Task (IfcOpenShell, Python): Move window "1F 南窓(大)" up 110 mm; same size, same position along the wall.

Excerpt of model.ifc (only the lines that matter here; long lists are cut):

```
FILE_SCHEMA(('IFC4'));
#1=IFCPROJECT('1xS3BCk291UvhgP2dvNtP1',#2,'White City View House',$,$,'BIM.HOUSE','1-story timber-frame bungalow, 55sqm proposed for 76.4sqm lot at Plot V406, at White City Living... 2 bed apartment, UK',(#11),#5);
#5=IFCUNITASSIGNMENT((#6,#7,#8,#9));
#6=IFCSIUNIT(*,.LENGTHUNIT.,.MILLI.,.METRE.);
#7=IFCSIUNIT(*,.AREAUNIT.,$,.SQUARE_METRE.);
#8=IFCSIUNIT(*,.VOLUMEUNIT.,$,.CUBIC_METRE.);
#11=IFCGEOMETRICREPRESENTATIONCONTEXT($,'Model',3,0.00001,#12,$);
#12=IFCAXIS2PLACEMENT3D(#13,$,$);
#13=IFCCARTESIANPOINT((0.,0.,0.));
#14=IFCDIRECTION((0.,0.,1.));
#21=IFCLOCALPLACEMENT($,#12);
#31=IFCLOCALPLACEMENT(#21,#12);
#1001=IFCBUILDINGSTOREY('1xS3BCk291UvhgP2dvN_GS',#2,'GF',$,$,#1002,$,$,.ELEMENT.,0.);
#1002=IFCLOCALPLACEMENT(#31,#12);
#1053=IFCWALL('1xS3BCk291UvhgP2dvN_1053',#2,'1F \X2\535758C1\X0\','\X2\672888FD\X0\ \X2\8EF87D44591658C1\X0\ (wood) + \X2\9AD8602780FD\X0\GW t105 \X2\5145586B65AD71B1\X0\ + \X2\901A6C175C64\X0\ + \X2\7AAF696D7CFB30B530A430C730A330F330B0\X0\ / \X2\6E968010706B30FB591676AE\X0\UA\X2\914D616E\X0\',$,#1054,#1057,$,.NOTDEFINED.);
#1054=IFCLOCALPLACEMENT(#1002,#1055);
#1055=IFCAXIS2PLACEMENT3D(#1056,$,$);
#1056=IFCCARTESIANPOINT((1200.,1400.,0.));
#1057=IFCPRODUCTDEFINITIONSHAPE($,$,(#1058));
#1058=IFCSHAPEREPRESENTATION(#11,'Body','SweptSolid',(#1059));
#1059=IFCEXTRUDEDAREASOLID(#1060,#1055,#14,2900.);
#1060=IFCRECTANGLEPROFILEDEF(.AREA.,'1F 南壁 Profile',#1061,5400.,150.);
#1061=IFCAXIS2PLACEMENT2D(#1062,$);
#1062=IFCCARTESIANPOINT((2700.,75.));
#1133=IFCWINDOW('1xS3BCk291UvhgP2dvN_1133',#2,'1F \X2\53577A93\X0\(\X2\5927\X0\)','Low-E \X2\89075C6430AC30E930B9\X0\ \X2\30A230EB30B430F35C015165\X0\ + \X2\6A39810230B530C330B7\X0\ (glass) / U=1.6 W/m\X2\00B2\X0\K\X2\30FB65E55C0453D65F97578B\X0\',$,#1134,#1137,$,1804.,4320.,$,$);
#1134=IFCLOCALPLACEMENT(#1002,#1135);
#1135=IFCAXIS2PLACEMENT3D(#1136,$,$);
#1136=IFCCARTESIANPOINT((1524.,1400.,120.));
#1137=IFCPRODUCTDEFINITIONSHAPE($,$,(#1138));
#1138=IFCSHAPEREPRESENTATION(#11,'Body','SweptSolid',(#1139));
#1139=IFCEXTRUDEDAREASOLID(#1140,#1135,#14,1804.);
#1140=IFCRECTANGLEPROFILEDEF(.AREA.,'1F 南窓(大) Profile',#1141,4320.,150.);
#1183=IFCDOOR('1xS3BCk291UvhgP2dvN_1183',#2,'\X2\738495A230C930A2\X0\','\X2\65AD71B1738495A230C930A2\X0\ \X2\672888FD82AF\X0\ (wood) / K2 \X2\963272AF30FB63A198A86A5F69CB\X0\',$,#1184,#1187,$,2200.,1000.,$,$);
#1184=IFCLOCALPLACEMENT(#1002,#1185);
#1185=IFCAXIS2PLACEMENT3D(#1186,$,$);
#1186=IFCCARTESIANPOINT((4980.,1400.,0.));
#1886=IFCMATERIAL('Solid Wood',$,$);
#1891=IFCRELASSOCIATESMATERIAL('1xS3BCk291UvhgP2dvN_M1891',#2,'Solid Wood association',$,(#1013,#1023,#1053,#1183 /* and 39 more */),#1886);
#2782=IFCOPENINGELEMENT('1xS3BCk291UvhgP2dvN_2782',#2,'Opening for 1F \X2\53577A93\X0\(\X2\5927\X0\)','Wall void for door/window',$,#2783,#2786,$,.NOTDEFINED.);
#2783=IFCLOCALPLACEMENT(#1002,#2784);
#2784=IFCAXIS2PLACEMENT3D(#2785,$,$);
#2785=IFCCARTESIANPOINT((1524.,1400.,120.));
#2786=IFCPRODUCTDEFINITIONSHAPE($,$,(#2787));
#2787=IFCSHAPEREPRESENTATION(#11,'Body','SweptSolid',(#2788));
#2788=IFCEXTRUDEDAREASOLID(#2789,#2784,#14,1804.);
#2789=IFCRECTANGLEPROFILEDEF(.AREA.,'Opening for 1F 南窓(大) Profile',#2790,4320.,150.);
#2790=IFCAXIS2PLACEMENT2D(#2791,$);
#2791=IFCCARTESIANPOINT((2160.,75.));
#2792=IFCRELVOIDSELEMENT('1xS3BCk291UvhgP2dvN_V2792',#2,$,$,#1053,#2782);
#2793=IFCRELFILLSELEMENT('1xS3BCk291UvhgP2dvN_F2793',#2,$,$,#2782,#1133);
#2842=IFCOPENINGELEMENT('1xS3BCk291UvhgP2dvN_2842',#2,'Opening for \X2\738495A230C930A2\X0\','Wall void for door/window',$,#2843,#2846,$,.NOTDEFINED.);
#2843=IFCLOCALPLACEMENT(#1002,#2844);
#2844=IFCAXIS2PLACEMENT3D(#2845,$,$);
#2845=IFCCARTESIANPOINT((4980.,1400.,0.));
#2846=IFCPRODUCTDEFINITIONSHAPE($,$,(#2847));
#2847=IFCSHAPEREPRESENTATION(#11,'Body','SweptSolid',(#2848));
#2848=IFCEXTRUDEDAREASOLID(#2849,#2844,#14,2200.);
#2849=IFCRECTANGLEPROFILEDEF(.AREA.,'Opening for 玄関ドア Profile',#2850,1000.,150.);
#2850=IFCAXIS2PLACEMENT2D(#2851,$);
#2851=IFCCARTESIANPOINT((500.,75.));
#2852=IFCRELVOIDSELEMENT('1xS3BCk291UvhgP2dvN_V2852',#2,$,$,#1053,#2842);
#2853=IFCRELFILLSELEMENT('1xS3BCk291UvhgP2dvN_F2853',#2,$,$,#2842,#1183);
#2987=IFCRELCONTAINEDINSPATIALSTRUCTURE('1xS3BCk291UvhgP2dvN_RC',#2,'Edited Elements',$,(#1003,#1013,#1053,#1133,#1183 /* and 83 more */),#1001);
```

```python
import numpy as np
import ifcopenshell
import ifcopenshell.api.geometry
import ifcopenshell.util.placement
import ifcopenshell.util.unit

model = ifcopenshell.open("model.ifc")
unit_scale = ifcopenshell.util.unit.calculate_unit_scale(model)

window = model.by_id(1133)
opening = window.FillsVoids[0].RelatingOpeningElement
dz = 0.11 / unit_scale

shift = np.array([0.0, 0.0, dz])
# The window is not placed relative to its opening, so move both.
for product in (opening, window):
    matrix = ifcopenshell.util.placement.get_local_placement(product.ObjectPlacement)
    matrix[:3, 3] += shift
    ifcopenshell.api.geometry.edit_object_placement(model, product=product, matrix=matrix, is_si=False)

print(f"moved by {dz * unit_scale:+.3f} m")

model.write("model_edited.ifc")
```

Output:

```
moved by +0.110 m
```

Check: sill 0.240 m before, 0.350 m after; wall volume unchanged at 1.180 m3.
